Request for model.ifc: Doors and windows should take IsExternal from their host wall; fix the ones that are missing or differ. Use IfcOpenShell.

First a look at what the model holds.

```python
import ifcopenshell
import ifcopenshell.util.element

model = ifcopenshell.open("model.ifc")
print(model.schema)
seen = {}
for e in model.by_type("IfcDoor") + model.by_type("IfcWindow"):
    if not e.FillsVoids:
        continue
    host = e.FillsVoids[0].RelatingOpeningElement.VoidsElements[0].RelatingBuildingElement
    own = ifcopenshell.util.element.get_pset(e, f"Pset_{e.is_a()[3:].removesuffix('StandardCase')}Common", "IsExternal")
    wall = ifcopenshell.util.element.get_pset(host, "Pset_WallCommon", "IsExternal")
    seen[e.is_a(), own, wall] = seen.get((e.is_a(), own, wall), 0) + 1
for (cls, own, wall), count in sorted(seen.items(), key=str):
    print(count, cls, "IsExternal:", own, "| host wall:", wall)
```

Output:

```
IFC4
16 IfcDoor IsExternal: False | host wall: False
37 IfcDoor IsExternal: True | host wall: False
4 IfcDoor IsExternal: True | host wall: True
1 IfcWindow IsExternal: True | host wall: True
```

```python
import ifcopenshell
import ifcopenshell.api.pset
import ifcopenshell.util.element

model = ifcopenshell.open("model.ifc")

count = 0
for ifc_class, pset_name in (("IfcDoor", "Pset_DoorCommon"), ("IfcWindow", "Pset_WindowCommon")):
    for e in model.by_type(ifc_class):
        if not e.FillsVoids:
            continue
        host = e.FillsVoids[0].RelatingOpeningElement.VoidsElements[0].RelatingBuildingElement
        external = ifcopenshell.util.element.get_pset(host, "Pset_WallCommon", "IsExternal")
        if external is None or ifcopenshell.util.element.get_pset(e, pset_name, "IsExternal") == external:
            continue
        pset = ifcopenshell.api.pset.add_pset(model, product=e, name=pset_name)
        ifcopenshell.api.pset.edit_pset(model, pset=pset, properties={"IsExternal": external})
        count += 1

print(count, "updated")

model.write("model_edited.ifc")
```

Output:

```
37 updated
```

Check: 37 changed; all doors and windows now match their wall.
